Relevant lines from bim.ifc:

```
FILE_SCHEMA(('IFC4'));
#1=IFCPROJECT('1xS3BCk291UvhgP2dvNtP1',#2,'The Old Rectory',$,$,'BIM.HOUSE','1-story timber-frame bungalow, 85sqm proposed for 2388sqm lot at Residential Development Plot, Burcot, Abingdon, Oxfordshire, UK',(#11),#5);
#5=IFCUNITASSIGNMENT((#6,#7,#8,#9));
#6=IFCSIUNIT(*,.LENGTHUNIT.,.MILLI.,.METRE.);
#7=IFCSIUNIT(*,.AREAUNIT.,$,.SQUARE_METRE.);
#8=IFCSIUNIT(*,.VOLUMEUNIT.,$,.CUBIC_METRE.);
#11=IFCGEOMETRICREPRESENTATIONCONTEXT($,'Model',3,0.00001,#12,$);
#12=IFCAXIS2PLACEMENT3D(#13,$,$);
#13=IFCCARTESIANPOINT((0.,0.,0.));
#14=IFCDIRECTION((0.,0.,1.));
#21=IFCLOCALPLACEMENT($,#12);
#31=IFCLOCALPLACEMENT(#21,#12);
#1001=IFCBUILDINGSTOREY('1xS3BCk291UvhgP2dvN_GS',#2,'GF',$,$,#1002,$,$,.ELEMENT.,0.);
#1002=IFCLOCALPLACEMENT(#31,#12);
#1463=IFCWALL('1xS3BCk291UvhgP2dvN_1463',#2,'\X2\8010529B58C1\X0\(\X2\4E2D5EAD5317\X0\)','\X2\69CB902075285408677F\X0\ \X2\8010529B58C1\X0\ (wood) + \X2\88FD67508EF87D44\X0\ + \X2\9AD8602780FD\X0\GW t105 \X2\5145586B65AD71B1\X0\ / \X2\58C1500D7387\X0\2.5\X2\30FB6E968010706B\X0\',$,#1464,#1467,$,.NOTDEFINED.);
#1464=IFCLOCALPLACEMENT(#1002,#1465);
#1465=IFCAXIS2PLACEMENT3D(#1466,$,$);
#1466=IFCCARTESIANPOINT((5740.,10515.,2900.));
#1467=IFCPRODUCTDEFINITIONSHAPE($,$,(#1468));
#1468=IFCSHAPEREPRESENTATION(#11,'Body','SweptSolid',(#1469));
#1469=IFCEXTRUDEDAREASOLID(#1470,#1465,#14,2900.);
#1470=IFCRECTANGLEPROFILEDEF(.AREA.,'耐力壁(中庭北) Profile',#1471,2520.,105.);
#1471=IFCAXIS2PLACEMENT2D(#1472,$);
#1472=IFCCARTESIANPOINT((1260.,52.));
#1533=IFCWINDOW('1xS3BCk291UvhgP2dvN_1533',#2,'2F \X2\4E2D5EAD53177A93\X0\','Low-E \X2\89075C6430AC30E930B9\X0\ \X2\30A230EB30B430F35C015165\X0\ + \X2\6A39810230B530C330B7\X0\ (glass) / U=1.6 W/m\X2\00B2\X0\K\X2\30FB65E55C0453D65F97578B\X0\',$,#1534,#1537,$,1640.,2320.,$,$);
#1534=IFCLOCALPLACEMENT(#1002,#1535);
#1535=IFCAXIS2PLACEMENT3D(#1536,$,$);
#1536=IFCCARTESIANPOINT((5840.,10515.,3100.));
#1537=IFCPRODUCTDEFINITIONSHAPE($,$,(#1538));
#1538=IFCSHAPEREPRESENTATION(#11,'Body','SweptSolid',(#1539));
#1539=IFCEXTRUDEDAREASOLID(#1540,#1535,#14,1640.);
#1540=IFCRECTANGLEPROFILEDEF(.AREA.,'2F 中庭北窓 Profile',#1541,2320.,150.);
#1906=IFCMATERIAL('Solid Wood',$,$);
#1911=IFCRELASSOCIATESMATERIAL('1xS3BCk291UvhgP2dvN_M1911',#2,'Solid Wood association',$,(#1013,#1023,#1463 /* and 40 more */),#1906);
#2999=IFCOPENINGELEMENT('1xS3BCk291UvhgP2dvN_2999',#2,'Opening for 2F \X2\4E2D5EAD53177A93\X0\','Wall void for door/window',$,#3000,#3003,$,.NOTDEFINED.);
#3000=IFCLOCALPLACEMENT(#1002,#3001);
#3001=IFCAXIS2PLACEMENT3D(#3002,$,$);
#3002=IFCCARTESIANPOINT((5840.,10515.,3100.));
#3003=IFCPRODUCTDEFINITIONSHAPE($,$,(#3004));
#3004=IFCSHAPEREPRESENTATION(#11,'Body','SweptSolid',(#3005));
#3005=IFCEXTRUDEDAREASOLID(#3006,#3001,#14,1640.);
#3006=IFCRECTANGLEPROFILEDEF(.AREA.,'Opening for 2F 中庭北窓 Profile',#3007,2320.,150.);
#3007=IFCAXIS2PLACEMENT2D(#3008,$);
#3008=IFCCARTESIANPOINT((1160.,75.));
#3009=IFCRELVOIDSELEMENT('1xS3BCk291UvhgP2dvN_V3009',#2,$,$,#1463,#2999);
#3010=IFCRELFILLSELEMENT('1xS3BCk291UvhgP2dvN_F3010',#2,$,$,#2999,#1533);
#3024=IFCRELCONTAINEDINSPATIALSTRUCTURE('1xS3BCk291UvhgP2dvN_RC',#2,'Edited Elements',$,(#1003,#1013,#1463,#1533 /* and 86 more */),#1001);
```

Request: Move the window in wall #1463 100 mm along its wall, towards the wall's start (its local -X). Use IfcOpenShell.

```python
import ifcopenshell
import ifcopenshell.api.geometry
import ifcopenshell.util.placement

model = ifcopenshell.open("bim.ifc")

window = model.by_id(1533)
opening = window.FillsVoids[0].RelatingOpeningElement
wall = opening.VoidsElements[0].RelatingBuildingElement

wall_matrix = ifcopenshell.util.placement.get_local_placement(wall.ObjectPlacement)
shift = wall_matrix[:3, 0] * -100.0
before = ifcopenshell.util.placement.get_local_placement(window.ObjectPlacement)[:3, 3].copy()

# The window is not placed relative to its opening, so move both.
for product in (opening, window):
    matrix = ifcopenshell.util.placement.get_local_placement(product.ObjectPlacement)
    matrix[:3, 3] += shift
    ifcopenshell.api.geometry.edit_object_placement(model, product=product, matrix=matrix, is_si=False)

after = ifcopenshell.util.placement.get_local_placement(window.ObjectPlacement)[:3, 3]
print("window moved by", (after - before).round(3) + 0.0)

model.write("bim_rev.ifc")
```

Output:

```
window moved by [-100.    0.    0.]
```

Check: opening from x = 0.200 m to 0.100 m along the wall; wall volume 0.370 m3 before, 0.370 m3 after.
